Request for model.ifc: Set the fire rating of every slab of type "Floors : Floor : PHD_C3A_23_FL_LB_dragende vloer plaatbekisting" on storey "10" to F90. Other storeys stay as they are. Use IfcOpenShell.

First a look at what the model holds.

```python
import ifcopenshell
import ifcopenshell.util.element

model = ifcopenshell.open("model.ifc")
print(model.schema)
storey = next(s for s in model.by_type("IfcBuildingStorey") if s.Name == "10")
slabs = [e for e in ifcopenshell.util.element.get_decomposition(storey) if e.is_a("IfcSlab")]
seen = {}
for e in slabs:
    element_type = ifcopenshell.util.element.get_type(e)
    key = (element_type.Name if element_type != e and element_type else None, ifcopenshell.util.element.get_pset(e, "Pset_SlabCommon", "FireRating"))
    seen[key] = seen.get(key, 0) + 1
for (name, value), count in sorted(seen.items(), key=str):
    print(count, "x", name, "|", value)
```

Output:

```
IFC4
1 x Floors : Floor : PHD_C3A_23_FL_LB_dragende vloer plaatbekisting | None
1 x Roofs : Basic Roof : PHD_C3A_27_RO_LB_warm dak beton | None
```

```python
import ifcopenshell
import ifcopenshell.api.pset
import ifcopenshell.util.element

model = ifcopenshell.open("model.ifc")

storey = next(s for s in model.by_type("IfcBuildingStorey") if s.Name == "10")
slabs = [e for e in ifcopenshell.util.element.get_decomposition(storey) if e.is_a("IfcSlab")]

count = 0
for e in slabs:
    element_type = ifcopenshell.util.element.get_type(e)
    if element_type in (None, e) or element_type.Name != "Floors : Floor : PHD_C3A_23_FL_LB_dragende vloer plaatbekisting":
        continue
    # add_pset returns the element's existing set when there is one.
    pset = ifcopenshell.api.pset.add_pset(model, product=e, name="Pset_SlabCommon")
    ifcopenshell.api.pset.edit_pset(model, pset=pset, properties={"FireRating": "F90"})
    count += 1

print(count, "slabs updated")

model.write("model_v2.ifc")
```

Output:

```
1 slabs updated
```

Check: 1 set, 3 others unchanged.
